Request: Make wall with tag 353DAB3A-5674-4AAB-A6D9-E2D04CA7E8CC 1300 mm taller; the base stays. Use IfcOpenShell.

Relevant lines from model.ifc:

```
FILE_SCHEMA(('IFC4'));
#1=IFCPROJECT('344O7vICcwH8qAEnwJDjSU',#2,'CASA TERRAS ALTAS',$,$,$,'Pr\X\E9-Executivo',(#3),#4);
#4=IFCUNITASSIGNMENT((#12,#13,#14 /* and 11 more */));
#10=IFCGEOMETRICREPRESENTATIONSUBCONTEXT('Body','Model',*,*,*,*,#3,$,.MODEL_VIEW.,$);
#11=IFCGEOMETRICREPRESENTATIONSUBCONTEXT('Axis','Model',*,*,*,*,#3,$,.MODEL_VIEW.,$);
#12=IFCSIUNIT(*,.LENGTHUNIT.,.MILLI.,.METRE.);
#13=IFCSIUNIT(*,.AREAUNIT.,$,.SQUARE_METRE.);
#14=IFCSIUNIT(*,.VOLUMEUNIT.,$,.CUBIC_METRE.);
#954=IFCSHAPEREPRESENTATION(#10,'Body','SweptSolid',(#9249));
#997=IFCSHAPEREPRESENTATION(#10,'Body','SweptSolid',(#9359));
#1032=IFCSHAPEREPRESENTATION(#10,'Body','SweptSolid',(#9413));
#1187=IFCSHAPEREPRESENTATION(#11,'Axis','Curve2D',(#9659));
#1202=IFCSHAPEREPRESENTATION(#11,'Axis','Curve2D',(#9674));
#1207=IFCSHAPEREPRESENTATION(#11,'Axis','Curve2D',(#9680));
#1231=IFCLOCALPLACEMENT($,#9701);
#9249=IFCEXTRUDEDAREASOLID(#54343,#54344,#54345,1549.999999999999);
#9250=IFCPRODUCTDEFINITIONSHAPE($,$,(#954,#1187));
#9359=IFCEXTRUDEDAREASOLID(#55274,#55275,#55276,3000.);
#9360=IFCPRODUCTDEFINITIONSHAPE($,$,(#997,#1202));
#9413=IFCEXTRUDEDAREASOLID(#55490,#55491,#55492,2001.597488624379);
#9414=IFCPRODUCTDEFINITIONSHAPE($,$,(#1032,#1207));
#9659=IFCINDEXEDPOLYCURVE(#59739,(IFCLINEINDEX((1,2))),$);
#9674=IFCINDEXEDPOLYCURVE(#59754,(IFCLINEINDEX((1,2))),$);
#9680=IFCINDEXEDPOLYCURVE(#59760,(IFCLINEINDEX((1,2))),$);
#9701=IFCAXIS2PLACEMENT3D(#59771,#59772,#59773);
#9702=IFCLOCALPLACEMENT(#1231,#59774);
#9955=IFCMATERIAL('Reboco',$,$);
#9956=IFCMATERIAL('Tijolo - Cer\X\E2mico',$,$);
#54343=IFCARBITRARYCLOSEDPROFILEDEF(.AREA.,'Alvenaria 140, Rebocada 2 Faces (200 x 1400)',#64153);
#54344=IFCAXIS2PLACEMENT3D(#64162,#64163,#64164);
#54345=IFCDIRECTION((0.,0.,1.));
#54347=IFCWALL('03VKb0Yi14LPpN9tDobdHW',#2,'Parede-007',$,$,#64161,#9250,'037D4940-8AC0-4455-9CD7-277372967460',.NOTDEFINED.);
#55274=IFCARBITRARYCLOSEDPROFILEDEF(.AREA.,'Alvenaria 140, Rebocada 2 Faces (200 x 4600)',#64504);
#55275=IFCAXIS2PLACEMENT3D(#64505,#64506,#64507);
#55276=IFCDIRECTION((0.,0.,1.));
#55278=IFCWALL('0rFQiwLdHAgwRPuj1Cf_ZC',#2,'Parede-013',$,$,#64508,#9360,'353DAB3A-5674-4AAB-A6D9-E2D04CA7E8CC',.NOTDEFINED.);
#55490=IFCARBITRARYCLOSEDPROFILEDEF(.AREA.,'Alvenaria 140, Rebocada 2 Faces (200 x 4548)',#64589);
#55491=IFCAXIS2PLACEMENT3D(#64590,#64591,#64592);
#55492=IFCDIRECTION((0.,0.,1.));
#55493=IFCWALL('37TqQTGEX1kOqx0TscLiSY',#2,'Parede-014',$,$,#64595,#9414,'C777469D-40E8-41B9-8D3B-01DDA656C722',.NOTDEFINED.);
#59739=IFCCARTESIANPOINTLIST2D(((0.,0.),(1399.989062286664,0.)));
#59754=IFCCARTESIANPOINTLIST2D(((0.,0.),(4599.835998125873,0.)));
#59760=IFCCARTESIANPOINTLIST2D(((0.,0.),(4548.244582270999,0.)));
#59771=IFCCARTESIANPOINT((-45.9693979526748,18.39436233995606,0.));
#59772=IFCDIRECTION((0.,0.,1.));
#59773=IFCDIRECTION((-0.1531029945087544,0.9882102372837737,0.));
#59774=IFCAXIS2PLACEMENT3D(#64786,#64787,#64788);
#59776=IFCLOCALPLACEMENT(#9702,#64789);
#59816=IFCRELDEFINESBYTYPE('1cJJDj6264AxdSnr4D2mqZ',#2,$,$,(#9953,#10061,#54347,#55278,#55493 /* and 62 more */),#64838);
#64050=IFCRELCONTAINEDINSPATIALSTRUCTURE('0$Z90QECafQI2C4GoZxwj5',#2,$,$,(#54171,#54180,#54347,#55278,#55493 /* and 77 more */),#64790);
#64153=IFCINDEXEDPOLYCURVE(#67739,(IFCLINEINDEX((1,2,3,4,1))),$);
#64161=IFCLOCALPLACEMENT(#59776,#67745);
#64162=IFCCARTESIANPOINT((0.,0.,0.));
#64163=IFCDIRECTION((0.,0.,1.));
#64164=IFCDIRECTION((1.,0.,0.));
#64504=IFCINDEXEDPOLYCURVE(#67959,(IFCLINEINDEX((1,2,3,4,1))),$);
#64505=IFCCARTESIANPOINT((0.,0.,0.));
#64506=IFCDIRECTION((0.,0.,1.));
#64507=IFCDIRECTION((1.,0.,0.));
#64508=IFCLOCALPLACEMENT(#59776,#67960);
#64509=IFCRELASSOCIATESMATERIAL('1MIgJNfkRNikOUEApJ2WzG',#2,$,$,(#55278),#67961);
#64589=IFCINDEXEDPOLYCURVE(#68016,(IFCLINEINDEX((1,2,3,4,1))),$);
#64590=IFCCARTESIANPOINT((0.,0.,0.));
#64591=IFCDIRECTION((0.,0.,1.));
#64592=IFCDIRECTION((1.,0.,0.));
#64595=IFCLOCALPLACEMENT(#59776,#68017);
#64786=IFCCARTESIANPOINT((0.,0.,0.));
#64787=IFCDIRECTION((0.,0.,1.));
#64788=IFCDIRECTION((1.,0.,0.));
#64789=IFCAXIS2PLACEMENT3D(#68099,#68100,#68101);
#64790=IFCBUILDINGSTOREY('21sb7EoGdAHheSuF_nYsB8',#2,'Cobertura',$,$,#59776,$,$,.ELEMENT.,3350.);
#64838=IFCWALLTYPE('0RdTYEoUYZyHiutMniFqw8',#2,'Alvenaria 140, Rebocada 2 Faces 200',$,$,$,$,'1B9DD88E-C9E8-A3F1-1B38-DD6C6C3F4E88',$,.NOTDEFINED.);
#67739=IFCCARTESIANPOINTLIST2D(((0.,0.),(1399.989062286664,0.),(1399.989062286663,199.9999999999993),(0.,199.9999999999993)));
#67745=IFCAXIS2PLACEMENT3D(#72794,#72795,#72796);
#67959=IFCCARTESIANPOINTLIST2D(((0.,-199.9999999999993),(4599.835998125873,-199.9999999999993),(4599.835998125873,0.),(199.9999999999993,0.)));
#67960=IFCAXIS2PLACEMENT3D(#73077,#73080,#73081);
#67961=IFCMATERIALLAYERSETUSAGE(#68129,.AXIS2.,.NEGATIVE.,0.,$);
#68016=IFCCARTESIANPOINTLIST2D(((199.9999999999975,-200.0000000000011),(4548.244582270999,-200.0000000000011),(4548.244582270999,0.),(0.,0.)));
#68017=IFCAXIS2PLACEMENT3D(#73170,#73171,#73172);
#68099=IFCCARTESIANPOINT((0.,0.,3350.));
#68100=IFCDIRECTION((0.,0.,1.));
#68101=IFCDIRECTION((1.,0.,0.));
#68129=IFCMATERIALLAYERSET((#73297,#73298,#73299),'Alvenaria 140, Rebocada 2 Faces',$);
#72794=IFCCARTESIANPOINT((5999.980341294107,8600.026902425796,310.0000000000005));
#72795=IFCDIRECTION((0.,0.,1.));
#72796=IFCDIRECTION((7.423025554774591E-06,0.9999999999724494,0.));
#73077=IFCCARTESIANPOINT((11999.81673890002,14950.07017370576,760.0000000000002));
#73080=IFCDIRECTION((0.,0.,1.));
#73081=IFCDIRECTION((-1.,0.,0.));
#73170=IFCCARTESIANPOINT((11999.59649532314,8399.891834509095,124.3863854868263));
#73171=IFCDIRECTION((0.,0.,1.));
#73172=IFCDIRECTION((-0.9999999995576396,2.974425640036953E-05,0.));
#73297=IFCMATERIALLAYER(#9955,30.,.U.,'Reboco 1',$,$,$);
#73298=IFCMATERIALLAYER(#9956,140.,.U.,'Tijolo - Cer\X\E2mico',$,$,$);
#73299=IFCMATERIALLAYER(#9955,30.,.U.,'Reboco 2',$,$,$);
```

```python
import ifcopenshell
import ifcopenshell.geom
import ifcopenshell.util.representation
import ifcopenshell.util.shape

model = ifcopenshell.open("model.ifc")
settings = ifcopenshell.geom.settings()


def volume(element):
    """Net volume in cubic metres, openings subtracted."""
    shape = ifcopenshell.geom.create_shape(settings, element)
    return ifcopenshell.util.shape.get_volume(shape.geometry)


wall = model.by_guid("0rFQiwLdHAgwRPuj1Cf_ZC")
before = volume(wall)

body = ifcopenshell.util.representation.get_representation(wall, "Model", "Body")
solid = body.Items[0]
old_height = solid.Depth
solid.Depth += 1300.0
after = volume(wall)

print(f"height {old_height:g} -> {solid.Depth:g}, volume {before:.3f} -> {after:.3f} m3")

model.write("model_updated.ifc")
```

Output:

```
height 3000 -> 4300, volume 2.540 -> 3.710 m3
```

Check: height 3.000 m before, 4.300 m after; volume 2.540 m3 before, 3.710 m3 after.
